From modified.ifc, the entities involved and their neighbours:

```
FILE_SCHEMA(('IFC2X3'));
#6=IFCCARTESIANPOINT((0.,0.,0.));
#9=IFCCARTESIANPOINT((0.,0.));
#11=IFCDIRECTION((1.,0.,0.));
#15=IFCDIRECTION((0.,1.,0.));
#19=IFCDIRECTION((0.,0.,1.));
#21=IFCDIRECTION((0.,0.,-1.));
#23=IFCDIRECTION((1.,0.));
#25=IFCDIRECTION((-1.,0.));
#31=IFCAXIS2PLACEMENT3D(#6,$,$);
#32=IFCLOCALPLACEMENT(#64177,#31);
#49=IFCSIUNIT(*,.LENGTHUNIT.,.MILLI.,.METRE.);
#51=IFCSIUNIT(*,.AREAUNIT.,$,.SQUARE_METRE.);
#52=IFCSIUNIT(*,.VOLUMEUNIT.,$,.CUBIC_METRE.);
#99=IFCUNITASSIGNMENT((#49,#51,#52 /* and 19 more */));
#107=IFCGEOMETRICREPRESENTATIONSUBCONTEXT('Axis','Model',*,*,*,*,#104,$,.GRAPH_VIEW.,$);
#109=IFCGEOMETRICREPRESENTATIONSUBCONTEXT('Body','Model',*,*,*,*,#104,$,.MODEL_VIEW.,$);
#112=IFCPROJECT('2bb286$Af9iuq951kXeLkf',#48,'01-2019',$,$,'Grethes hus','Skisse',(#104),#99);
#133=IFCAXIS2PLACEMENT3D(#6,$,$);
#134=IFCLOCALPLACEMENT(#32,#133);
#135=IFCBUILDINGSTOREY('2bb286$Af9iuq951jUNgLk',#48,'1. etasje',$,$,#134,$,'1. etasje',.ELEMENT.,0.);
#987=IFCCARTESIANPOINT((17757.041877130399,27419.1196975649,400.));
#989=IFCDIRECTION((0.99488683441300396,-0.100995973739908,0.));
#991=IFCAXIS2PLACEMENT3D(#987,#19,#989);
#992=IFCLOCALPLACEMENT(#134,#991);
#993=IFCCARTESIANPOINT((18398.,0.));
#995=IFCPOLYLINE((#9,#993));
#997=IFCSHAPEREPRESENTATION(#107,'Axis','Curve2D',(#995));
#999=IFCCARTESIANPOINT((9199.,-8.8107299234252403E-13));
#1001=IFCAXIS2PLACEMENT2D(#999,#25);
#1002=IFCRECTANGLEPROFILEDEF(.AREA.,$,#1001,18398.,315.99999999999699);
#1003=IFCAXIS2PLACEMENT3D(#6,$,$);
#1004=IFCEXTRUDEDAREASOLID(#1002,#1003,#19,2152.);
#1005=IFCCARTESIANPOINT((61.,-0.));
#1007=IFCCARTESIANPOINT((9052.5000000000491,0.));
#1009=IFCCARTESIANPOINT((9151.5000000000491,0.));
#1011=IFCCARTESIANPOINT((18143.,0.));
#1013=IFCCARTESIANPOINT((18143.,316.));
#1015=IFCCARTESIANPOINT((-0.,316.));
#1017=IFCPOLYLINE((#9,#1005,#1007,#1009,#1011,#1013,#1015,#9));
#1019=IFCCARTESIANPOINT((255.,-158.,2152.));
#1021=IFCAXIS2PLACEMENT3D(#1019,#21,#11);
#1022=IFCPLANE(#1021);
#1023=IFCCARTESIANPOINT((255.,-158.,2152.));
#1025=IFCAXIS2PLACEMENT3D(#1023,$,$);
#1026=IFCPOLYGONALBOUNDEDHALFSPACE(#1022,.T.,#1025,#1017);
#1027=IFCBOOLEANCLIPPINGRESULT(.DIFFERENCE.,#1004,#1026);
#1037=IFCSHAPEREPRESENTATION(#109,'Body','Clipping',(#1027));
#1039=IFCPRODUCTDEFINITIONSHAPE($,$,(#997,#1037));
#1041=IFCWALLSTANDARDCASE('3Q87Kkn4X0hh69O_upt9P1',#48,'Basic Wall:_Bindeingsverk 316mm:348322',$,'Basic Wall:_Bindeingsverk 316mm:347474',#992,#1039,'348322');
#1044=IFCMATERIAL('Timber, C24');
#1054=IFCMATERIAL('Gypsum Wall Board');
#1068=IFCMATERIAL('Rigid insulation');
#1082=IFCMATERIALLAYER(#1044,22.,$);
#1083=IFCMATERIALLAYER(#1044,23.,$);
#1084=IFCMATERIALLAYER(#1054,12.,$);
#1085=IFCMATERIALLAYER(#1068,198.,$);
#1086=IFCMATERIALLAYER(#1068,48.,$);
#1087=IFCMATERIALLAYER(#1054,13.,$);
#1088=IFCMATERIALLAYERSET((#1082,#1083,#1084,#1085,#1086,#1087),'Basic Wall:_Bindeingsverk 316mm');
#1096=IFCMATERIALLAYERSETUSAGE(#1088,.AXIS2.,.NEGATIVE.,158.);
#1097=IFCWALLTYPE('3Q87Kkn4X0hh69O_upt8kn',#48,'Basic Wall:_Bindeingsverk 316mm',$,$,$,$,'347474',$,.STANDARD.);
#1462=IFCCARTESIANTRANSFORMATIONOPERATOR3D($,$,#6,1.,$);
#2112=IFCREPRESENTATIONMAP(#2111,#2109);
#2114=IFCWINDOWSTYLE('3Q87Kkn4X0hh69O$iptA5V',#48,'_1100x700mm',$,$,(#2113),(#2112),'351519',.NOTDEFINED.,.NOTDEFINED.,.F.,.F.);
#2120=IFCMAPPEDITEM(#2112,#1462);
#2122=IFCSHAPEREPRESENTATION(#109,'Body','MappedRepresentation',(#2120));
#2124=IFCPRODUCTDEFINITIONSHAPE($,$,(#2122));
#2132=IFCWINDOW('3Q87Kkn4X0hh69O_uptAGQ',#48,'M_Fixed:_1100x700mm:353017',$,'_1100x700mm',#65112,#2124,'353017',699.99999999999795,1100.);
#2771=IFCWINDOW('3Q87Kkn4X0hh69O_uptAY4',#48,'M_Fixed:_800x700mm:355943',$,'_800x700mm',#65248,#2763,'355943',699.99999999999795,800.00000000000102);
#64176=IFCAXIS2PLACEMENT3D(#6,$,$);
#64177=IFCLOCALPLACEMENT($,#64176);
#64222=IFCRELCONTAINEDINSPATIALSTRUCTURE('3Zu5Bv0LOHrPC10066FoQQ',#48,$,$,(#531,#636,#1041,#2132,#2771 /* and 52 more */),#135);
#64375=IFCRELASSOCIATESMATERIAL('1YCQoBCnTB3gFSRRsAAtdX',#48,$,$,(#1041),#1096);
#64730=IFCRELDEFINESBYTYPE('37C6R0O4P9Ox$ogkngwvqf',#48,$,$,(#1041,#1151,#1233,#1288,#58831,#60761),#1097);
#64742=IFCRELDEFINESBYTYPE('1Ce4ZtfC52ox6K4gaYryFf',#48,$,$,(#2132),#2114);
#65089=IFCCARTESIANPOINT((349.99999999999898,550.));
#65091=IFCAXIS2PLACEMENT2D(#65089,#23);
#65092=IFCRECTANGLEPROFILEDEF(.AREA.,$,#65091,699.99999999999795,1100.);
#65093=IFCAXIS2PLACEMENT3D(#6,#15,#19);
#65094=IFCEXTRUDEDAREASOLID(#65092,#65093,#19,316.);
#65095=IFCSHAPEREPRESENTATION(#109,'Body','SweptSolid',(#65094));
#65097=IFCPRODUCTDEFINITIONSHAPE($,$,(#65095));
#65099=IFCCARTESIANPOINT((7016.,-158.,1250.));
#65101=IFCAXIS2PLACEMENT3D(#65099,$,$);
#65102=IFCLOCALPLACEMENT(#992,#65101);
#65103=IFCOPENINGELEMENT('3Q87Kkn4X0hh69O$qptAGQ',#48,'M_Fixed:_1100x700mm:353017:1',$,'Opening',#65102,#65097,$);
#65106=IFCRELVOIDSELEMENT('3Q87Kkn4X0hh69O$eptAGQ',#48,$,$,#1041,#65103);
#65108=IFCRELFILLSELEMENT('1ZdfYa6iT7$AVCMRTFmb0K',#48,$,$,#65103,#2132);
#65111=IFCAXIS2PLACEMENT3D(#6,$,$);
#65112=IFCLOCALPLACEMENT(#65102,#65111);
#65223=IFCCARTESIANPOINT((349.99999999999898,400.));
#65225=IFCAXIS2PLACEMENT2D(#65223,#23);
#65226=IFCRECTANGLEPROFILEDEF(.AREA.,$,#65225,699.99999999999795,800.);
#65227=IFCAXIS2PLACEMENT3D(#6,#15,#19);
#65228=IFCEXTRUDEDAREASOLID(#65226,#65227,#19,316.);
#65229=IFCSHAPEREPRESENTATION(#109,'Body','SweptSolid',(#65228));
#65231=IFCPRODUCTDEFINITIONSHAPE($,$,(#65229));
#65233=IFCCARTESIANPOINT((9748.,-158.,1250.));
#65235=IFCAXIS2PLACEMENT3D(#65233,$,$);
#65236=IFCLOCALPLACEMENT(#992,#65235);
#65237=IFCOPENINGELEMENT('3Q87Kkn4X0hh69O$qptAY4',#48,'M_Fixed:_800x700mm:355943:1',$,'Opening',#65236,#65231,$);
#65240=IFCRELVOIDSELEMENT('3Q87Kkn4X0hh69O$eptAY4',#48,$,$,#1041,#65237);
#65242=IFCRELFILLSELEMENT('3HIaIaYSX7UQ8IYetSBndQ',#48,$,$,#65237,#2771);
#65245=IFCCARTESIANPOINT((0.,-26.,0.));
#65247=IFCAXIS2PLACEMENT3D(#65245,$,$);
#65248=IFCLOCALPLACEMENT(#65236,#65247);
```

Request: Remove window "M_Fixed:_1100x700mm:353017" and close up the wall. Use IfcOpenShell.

```python
import ifcopenshell
import ifcopenshell.api.feature
import ifcopenshell.api.root
import ifcopenshell.geom
import ifcopenshell.util.shape

model = ifcopenshell.open("modified.ifc")
settings = ifcopenshell.geom.settings()


def volume(element):
    """Net volume in cubic metres, openings subtracted."""
    shape = ifcopenshell.geom.create_shape(settings, element)
    return ifcopenshell.util.shape.get_volume(shape.geometry)


window = model.by_guid("3Q87Kkn4X0hh69O_uptAGQ")
opening = window.FillsVoids[0].RelatingOpeningElement
wall = opening.VoidsElements[0].RelatingBuildingElement
before = volume(wall)

ifcopenshell.api.root.remove_product(model, product=window)
ifcopenshell.api.feature.remove_feature(model, feature=opening)

after = volume(wall)

print(f"wall volume {before:.3f} -> {after:.3f} m3")

model.write("modified_updated.ifc")
```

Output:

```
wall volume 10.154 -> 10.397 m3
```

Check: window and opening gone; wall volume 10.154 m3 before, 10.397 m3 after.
